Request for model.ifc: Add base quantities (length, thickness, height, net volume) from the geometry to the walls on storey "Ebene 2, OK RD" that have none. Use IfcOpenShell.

First a look at what the model holds.

```python
import ifcopenshell
import ifcopenshell.util.element
import ifcopenshell.util.unit

model = ifcopenshell.open("model.ifc")
print(model.schema)
for unit_type in ("LENGTHUNIT", "AREAUNIT", "VOLUMEUNIT"):
    print(unit_type, ifcopenshell.util.unit.calculate_unit_scale(model, unit_type))
storey = next(s for s in model.by_type("IfcBuildingStorey") if s.Name == "Ebene 2, OK RD")
walls = [e for e in ifcopenshell.util.element.get_decomposition(storey) if e.is_a("IfcWall")]
for e in sorted(walls, key=lambda e: e.id()):
    print(e.id(), e.is_a(), e.Name, list(ifcopenshell.util.element.get_psets(e, qtos_only=True)), sep=" | ")
```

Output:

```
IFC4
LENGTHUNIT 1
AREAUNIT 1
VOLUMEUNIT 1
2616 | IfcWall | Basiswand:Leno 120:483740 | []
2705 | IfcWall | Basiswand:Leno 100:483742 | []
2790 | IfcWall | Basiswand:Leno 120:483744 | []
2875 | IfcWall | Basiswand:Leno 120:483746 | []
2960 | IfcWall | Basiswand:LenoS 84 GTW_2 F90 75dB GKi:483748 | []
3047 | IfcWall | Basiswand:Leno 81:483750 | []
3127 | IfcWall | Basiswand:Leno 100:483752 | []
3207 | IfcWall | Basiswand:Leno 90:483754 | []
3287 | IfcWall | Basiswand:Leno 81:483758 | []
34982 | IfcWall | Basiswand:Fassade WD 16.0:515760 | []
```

```python
import ifcopenshell
import ifcopenshell.api.pset
import ifcopenshell.geom
import ifcopenshell.util.element
import ifcopenshell.util.shape
import ifcopenshell.util.unit

model = ifcopenshell.open("model.ifc")
unit_scale = ifcopenshell.util.unit.calculate_unit_scale(model)
volume_scale = ifcopenshell.util.unit.calculate_unit_scale(model, "VOLUMEUNIT")
settings = ifcopenshell.geom.settings()

storey = next(s for s in model.by_type("IfcBuildingStorey") if s.Name == "Ebene 2, OK RD")
walls = [e for e in ifcopenshell.util.element.get_decomposition(storey) if e.is_a("IfcWall")]

for e in sorted(walls, key=lambda e: e.id()):
    if ifcopenshell.util.element.get_psets(e, qtos_only=True, should_inherit=False):
        continue
    # Geometry comes back in metres, in the element's own axes.
    shape = ifcopenshell.geom.create_shape(settings, e)
    values = {
        "Length": ifcopenshell.util.shape.get_x(shape.geometry) / unit_scale,
        "Width": ifcopenshell.util.shape.get_y(shape.geometry) / unit_scale,
        "Height": ifcopenshell.util.shape.get_z(shape.geometry) / unit_scale,
        "NetVolume": ifcopenshell.util.shape.get_volume(shape.geometry) / volume_scale,
    }
    qto = ifcopenshell.api.pset.add_qto(model, product=e, name="Qto_WallBaseQuantities")
    ifcopenshell.api.pset.edit_qto(model, qto=qto, properties=values)
    print(e.id(), {k: round(v, 3) for k, v in values.items()})

model.write("model_edited.ifc")
```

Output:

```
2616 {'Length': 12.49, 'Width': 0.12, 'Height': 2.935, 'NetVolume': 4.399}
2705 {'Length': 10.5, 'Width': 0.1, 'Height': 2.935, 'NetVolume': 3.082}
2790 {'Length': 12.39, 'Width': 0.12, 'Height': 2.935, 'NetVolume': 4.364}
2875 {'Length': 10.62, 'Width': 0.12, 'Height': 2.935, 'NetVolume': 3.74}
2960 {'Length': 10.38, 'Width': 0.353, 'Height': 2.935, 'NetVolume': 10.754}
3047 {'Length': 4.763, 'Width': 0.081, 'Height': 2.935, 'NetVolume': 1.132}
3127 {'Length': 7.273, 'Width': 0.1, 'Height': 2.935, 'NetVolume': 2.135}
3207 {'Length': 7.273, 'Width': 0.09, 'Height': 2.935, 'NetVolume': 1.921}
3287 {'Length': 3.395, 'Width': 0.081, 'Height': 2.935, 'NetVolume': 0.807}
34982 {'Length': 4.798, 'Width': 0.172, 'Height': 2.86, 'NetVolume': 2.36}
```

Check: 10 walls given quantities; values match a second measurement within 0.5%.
